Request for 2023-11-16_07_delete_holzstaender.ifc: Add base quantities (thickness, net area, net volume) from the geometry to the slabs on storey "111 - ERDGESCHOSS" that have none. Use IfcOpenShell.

First a look at what the model holds.

```python
import ifcopenshell
import ifcopenshell.util.element
import ifcopenshell.util.unit

model = ifcopenshell.open("2023-11-16_07_delete_holzstaender.ifc")
print(model.schema)
for unit_type in ("LENGTHUNIT", "AREAUNIT", "VOLUMEUNIT"):
    print(unit_type, ifcopenshell.util.unit.calculate_unit_scale(model, unit_type))
storey = next(s for s in model.by_type("IfcBuildingStorey") if s.Name == "111 - ERDGESCHOSS")
slabs = [e for e in ifcopenshell.util.element.get_decomposition(storey) if e.is_a("IfcSlab")]
for e in sorted(slabs, key=lambda e: e.id()):
    print(e.id(), e.is_a(), e.Name, list(ifcopenshell.util.element.get_psets(e, qtos_only=True)), sep=" | ")
```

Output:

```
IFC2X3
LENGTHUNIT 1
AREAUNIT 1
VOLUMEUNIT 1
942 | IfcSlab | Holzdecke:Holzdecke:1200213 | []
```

```python
import ifcopenshell
import ifcopenshell.api.pset
import ifcopenshell.geom
import ifcopenshell.util.element
import ifcopenshell.util.shape
import ifcopenshell.util.unit

model = ifcopenshell.open("2023-11-16_07_delete_holzstaender.ifc")
unit_scale = ifcopenshell.util.unit.calculate_unit_scale(model)
area_scale = ifcopenshell.util.unit.calculate_unit_scale(model, "AREAUNIT")
volume_scale = ifcopenshell.util.unit.calculate_unit_scale(model, "VOLUMEUNIT")
settings = ifcopenshell.geom.settings()

storey = next(s for s in model.by_type("IfcBuildingStorey") if s.Name == "111 - ERDGESCHOSS")
slabs = [e for e in ifcopenshell.util.element.get_decomposition(storey) if e.is_a("IfcSlab")]

for e in sorted(slabs, key=lambda e: e.id()):
    if ifcopenshell.util.element.get_psets(e, qtos_only=True, should_inherit=False):
        continue
    # Geometry comes back in metres, in the element's own axes.
    shape = ifcopenshell.geom.create_shape(settings, e)
    values = {
        "Width": ifcopenshell.util.shape.get_z(shape.geometry) / unit_scale,
        "NetArea": ifcopenshell.util.shape.get_footprint_area(shape.geometry) / area_scale,
        "NetVolume": ifcopenshell.util.shape.get_volume(shape.geometry) / volume_scale,
    }
    qto = ifcopenshell.api.pset.add_qto(model, product=e, name="BaseQuantities")
    ifcopenshell.api.pset.edit_qto(model, qto=qto, properties=values)
    print(e.id(), {k: round(v, 3) for k, v in values.items()})

model.write("2023-11-16_07_delete_holzstaender_updated.ifc")
```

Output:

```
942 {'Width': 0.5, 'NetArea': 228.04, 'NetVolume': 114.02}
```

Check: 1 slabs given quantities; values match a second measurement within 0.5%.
